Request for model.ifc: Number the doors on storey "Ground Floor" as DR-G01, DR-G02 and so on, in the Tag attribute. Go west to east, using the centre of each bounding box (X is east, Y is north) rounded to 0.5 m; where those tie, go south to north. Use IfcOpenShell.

First a look at what the model holds.

```python
import ifcopenshell
import ifcopenshell.util.element
import ifcopenshell.util.placement

model = ifcopenshell.open("model.ifc")
print(model.schema)
storey = next(s for s in model.by_type("IfcBuildingStorey") if s.Name == "Ground Floor")
doors = [e for e in ifcopenshell.util.element.get_decomposition(storey) if e.is_a("IfcDoor")]
for e in sorted(doors, key=lambda e: e.id()):
    origin = ifcopenshell.util.placement.get_local_placement(e.ObjectPlacement)[:3, 3]
    print(e.id(), e.Tag, e.Name, origin.round(2) + 0.0, sep=" | ")
```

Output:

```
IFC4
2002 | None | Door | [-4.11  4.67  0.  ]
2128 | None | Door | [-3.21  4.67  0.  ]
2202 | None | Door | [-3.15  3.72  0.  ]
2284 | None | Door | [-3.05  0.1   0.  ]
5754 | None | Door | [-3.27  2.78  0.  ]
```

```python
import ifcopenshell
import ifcopenshell.geom
import ifcopenshell.util.element
import ifcopenshell.util.shape

model = ifcopenshell.open("model.ifc")
settings = ifcopenshell.geom.settings()
settings.set("use-world-coords", True)


def centre(element):
    shape = ifcopenshell.geom.create_shape(settings, element)
    return ifcopenshell.util.shape.get_bbox_centroid(shape.geometry)


storey = next(s for s in model.by_type("IfcBuildingStorey") if s.Name == "Ground Floor")
doors = [e for e in ifcopenshell.util.element.get_decomposition(storey) if e.is_a("IfcDoor")]

# Insertion points can sit at a corner or the storey origin, so sort by the geometry (in metres).
centres = {e: centre(e) for e in doors}
doors.sort(key=lambda e: (round(centres[e][0] / 0.5), centres[e][1]))

for i, e in enumerate(doors, start=1):
    number = f"DR-G{i:02d}"
    e.Tag = number
    print(e.id(), number)

model.write("model_rev.ifc")
```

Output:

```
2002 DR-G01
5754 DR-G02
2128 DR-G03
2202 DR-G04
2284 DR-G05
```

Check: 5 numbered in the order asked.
